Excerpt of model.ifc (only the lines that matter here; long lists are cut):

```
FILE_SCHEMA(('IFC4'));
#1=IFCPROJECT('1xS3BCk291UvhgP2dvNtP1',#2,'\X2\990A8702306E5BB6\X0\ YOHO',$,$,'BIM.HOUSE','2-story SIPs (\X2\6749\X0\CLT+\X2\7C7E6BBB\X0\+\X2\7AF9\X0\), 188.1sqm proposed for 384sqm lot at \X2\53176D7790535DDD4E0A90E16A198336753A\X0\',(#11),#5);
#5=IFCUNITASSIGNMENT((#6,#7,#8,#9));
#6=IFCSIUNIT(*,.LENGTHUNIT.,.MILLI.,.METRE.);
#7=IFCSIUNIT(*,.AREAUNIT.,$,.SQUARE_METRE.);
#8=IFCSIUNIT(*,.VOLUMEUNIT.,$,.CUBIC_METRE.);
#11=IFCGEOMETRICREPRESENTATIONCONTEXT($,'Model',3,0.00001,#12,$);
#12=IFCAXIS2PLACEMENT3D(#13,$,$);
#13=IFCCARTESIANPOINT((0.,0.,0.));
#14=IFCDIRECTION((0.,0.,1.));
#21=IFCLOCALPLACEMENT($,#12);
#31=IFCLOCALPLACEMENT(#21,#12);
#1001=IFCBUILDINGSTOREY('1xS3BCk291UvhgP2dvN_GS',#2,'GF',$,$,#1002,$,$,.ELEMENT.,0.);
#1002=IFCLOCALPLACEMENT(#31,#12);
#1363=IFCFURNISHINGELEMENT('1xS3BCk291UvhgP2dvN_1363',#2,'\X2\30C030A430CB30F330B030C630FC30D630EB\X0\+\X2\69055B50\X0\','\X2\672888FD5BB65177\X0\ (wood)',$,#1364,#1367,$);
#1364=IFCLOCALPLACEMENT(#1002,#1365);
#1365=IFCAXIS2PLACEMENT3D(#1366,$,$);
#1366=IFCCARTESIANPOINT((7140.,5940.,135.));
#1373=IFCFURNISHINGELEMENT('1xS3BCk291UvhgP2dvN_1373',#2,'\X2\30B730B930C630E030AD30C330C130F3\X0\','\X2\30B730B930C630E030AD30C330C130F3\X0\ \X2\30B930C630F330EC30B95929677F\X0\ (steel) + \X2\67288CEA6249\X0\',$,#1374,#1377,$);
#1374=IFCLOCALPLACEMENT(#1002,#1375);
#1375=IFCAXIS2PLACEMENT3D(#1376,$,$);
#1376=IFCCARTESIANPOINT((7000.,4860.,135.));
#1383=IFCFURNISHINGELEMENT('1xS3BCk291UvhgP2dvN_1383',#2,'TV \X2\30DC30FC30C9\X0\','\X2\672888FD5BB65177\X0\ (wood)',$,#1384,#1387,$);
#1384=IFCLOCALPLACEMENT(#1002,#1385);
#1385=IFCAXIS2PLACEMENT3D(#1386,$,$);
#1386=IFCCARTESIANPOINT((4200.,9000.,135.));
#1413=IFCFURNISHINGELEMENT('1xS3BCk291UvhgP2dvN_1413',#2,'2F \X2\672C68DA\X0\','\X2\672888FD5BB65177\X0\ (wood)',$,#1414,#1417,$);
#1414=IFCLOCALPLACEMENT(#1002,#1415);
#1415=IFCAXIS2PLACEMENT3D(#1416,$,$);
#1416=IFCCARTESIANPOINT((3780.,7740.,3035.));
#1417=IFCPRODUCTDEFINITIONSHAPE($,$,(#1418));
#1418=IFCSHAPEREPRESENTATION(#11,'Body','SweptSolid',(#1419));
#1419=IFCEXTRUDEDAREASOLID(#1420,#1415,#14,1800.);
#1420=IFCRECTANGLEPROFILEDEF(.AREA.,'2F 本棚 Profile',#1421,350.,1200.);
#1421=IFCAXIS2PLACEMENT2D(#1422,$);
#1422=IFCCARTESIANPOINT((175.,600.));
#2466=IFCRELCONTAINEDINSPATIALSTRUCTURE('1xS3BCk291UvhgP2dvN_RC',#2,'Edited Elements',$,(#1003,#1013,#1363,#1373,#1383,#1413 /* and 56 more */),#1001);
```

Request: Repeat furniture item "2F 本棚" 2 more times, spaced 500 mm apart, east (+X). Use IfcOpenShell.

```python
import numpy as np
import ifcopenshell
import ifcopenshell.api.geometry
import ifcopenshell.api.root
import ifcopenshell.util.element
import ifcopenshell.util.placement
import ifcopenshell.util.unit

model = ifcopenshell.open("model.ifc")
unit_scale = ifcopenshell.util.unit.calculate_unit_scale(model)


def reuse_history(source, copy):
    """copy_class also copies each property set's owner history, people and application; keep the originals."""
    for rel in copy.IsDefinedBy:
        if rel.is_a("IfcRelDefinesByProperties") and (history := rel.RelatingPropertyDefinition.OwnerHistory):
            rel.RelatingPropertyDefinition.OwnerHistory = source.OwnerHistory
            ifcopenshell.util.element.remove_deep2(model, history)


source = model.by_id(1413)
base = ifcopenshell.util.placement.get_local_placement(source.ObjectPlacement)
step = np.array([1.0, 0.0, 0.0]) * 0.5 / unit_scale

for i in range(1, 3):
    copy = ifcopenshell.api.root.copy_class(model, product=source)
    copy.Representation = ifcopenshell.util.element.copy_deep(
        model, source.Representation, exclude=["IfcGeometricRepresentationContext", "IfcRepresentationMap"]
    )
    reuse_history(source, copy)
    matrix = base.copy()
    matrix[:3, 3] += i * step
    print("added at", matrix[:3, 3].round(3) + 0.0)
    ifcopenshell.api.geometry.edit_object_placement(model, product=copy, matrix=matrix, is_si=False)

model.write("model-out.ifc")
```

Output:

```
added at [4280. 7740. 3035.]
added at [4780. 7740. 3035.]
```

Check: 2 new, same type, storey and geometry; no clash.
